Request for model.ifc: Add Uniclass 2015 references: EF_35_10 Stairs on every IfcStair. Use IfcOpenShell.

First a look at what the model holds.

```python
import ifcopenshell

model = ifcopenshell.open("model.ifc")
print(model.schema)
print("classifications:", [c.Name for c in model.by_type("IfcClassification")])
for ifc_class in ("IfcDoor", "IfcRoof", "IfcStair", "IfcWall", "IfcWindow"):
    print(ifc_class, len(model.by_type(ifc_class)))
```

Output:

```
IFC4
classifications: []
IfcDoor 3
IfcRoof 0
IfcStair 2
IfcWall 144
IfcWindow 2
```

```python
import ifcopenshell
import ifcopenshell.api.classification

model = ifcopenshell.open("model.ifc")

system = ifcopenshell.api.classification.add_classification(model, classification="Uniclass 2015")

codes = {
    "IfcStair": ("EF_35_10", "Stairs"),
}
for ifc_class, (code, name) in codes.items():
    products = model.by_type(ifc_class)
    ifcopenshell.api.classification.add_reference(
        model, products=products, classification=system, identification=code, name=name
    )
    print(code, len(products))

model.write("model_updated.ifc")
```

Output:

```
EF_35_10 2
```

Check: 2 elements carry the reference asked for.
